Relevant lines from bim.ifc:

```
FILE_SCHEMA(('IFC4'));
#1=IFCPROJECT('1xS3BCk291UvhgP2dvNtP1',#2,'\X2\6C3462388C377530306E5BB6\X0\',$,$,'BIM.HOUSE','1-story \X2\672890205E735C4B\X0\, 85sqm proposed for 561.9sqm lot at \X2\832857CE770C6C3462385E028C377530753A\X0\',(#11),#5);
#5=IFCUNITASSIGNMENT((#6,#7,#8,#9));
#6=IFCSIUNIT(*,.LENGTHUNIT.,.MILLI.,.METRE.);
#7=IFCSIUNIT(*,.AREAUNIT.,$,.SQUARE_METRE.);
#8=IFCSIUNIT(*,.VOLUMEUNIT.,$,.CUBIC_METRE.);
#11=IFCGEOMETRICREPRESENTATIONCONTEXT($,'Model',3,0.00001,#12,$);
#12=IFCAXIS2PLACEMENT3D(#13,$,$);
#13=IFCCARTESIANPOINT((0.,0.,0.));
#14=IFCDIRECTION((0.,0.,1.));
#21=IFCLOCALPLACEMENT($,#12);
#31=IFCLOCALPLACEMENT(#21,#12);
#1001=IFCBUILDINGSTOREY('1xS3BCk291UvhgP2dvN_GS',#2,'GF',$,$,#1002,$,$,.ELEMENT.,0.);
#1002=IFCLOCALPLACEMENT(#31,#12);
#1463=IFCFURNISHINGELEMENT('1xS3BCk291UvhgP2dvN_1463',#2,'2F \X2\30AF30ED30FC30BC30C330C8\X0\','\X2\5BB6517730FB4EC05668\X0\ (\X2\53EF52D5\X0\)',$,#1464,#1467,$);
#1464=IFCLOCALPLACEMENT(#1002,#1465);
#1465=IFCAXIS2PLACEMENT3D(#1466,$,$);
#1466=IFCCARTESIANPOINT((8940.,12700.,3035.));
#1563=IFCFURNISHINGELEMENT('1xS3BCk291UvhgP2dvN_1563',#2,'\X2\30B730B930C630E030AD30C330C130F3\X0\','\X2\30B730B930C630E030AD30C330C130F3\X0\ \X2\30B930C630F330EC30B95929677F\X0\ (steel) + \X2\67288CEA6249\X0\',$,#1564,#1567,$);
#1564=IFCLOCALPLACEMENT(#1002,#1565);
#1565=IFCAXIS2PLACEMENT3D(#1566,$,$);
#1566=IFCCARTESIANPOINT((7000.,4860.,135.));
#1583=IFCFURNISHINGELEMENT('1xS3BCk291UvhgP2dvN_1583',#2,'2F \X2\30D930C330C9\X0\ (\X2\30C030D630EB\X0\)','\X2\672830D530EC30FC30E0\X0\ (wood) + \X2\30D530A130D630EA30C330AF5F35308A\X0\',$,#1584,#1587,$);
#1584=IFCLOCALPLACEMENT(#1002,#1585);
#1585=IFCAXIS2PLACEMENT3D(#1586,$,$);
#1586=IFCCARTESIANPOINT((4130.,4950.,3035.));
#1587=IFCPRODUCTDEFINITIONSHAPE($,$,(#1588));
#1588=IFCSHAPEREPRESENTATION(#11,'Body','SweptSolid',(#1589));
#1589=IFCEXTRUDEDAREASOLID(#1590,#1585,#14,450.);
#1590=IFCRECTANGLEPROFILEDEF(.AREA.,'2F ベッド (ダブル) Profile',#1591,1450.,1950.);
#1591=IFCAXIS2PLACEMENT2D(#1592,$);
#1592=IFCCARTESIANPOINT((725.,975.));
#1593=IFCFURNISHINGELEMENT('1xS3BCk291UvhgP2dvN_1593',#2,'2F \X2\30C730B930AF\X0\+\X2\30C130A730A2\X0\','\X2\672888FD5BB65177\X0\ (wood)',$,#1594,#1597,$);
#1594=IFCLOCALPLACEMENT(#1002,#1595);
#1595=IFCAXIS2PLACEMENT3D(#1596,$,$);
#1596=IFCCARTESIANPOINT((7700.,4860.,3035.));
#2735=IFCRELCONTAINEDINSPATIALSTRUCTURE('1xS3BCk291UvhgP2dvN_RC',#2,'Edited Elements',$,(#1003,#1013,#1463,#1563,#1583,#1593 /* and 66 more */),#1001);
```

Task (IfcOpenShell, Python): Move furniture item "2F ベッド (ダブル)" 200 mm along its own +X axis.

```python
import ifcopenshell
import ifcopenshell.api.geometry
import ifcopenshell.util.placement

model = ifcopenshell.open("bim.ifc")

item = model.by_guid("1xS3BCk291UvhgP2dvN_1583")
matrix = ifcopenshell.util.placement.get_local_placement(item.ObjectPlacement)
matrix[:3, 3] += matrix[:3, 0] * 200.0
ifcopenshell.api.geometry.edit_object_placement(model, product=item, matrix=matrix, is_si=False)

print(ifcopenshell.util.placement.get_local_placement(item.ObjectPlacement).round(3) + 0.0)

model.write("bim_edited.ifc")
```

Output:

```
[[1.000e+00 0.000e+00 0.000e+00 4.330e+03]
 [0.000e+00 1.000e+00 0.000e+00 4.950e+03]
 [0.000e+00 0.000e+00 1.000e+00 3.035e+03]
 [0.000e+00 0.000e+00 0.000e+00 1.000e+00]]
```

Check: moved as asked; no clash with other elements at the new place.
